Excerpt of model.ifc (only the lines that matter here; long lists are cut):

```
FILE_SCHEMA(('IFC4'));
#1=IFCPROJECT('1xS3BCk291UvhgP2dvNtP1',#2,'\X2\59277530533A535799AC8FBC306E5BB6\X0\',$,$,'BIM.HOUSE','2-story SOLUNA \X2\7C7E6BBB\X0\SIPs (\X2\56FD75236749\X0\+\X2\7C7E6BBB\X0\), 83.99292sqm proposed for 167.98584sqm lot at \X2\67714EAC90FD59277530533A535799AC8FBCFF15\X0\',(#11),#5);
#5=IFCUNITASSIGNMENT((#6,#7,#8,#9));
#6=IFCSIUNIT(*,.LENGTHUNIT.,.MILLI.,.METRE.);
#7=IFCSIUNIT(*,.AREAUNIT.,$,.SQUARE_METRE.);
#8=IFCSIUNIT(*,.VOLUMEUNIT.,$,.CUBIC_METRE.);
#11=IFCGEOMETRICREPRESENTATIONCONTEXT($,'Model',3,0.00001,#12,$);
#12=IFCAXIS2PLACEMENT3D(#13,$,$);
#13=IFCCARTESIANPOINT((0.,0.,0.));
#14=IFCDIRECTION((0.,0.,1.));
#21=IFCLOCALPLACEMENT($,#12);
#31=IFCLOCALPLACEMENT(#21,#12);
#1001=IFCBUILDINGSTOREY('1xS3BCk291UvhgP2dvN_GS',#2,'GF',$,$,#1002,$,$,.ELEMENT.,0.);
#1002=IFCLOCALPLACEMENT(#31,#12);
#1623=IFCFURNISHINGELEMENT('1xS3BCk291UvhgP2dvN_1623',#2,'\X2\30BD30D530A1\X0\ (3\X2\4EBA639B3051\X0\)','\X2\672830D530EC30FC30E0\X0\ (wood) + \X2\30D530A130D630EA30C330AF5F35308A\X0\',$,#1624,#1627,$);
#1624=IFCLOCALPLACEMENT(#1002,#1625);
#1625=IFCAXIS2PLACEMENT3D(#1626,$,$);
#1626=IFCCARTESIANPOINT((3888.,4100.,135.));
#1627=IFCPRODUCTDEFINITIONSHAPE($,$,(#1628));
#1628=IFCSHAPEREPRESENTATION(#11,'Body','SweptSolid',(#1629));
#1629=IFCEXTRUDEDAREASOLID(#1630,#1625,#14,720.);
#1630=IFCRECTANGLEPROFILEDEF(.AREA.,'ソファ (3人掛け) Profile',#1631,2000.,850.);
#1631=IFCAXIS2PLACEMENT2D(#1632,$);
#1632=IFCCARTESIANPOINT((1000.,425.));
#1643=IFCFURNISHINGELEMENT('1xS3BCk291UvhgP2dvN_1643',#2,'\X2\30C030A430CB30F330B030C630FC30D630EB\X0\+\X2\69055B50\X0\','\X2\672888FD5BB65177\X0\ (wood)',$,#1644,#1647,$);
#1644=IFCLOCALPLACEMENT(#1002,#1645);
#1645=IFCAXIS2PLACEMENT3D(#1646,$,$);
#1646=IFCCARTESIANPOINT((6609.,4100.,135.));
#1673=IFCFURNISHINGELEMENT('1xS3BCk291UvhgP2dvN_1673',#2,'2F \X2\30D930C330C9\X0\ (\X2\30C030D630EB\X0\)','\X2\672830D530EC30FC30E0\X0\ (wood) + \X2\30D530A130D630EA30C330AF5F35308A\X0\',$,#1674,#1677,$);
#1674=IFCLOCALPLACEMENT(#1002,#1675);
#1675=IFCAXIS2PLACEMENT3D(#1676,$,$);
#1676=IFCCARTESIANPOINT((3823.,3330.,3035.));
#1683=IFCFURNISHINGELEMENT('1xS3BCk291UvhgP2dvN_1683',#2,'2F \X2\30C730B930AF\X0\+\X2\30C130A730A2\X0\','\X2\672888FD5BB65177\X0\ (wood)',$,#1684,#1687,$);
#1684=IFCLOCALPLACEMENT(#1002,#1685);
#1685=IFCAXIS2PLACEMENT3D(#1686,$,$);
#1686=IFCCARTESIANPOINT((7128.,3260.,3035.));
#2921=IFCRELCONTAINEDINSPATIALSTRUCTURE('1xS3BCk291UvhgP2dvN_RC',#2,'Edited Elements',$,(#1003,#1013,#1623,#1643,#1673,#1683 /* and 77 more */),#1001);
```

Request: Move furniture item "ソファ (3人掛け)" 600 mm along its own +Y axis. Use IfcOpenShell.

```python
import ifcopenshell
import ifcopenshell.api.geometry
import ifcopenshell.util.placement
import ifcopenshell.util.unit

model = ifcopenshell.open("model.ifc")
unit_scale = ifcopenshell.util.unit.calculate_unit_scale(model)

item = model.by_id(1623)
matrix = ifcopenshell.util.placement.get_local_placement(item.ObjectPlacement)
matrix[:3, 3] += matrix[:3, 1] * 0.6 / unit_scale
ifcopenshell.api.geometry.edit_object_placement(model, product=item, matrix=matrix, is_si=False)

print(ifcopenshell.util.placement.get_local_placement(item.ObjectPlacement).round(3) + 0.0)

model.write("model_v2.ifc")
```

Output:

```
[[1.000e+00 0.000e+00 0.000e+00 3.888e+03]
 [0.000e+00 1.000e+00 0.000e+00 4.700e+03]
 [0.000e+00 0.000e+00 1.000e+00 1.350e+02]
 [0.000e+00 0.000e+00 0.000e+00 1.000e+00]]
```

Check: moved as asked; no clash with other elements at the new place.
